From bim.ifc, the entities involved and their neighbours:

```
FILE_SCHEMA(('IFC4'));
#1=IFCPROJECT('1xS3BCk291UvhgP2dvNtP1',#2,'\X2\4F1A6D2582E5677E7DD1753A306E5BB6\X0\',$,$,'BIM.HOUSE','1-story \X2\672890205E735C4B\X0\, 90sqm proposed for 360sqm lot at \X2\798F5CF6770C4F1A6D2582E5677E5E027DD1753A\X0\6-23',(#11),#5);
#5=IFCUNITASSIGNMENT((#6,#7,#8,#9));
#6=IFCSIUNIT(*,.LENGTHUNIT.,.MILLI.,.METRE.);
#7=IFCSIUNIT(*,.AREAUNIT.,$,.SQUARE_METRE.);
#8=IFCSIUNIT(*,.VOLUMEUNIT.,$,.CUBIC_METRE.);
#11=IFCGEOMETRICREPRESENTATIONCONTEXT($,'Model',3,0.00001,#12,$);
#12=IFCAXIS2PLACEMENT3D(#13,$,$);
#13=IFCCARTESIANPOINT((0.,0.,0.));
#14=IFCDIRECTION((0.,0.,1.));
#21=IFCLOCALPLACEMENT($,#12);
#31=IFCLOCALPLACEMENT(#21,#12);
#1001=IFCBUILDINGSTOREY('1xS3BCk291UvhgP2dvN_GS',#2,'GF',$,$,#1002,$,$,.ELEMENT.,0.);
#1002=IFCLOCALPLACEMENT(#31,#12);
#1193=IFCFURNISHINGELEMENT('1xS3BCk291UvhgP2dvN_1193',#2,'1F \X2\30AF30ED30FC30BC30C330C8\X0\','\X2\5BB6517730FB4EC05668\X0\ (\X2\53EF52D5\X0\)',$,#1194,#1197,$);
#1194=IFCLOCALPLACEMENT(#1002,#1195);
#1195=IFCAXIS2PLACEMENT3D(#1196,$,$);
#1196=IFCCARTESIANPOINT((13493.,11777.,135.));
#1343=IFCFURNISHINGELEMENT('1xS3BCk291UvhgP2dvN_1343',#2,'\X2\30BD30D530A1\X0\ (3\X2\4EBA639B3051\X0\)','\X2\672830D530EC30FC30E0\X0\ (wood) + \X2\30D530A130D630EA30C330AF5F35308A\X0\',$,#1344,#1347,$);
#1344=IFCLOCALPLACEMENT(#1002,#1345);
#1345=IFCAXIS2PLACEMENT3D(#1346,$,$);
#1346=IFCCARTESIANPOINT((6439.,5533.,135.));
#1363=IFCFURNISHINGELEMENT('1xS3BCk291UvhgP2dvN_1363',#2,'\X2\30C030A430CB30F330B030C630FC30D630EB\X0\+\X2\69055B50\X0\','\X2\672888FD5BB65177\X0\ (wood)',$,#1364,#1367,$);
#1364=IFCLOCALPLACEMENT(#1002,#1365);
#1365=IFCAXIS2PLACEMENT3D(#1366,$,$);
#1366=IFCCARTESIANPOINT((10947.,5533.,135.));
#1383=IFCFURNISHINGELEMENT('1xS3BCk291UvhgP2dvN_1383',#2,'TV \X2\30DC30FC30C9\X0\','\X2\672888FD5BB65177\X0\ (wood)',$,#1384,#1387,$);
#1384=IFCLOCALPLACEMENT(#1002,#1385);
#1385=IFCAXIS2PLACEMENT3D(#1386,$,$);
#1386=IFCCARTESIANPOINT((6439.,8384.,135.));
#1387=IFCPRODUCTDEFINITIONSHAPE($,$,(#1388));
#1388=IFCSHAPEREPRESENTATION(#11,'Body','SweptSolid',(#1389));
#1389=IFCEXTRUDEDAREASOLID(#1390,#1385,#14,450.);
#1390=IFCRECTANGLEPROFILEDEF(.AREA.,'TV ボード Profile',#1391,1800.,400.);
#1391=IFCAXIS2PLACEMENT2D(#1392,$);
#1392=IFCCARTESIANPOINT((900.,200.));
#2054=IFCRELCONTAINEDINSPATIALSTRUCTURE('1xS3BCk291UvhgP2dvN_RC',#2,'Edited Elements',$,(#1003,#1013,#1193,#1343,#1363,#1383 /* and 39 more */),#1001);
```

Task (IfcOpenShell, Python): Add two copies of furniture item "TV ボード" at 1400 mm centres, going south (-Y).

```python
import numpy as np
import ifcopenshell
import ifcopenshell.api.geometry
import ifcopenshell.api.root
import ifcopenshell.util.element
import ifcopenshell.util.placement

model = ifcopenshell.open("bim.ifc")


def reuse_history(source, copy):
    """copy_class also copies each property set's owner history, people and application; keep the originals."""
    for rel in copy.IsDefinedBy:
        if rel.is_a("IfcRelDefinesByProperties") and (history := rel.RelatingPropertyDefinition.OwnerHistory):
            rel.RelatingPropertyDefinition.OwnerHistory = source.OwnerHistory
            ifcopenshell.util.element.remove_deep2(model, history)


source = model.by_guid("1xS3BCk291UvhgP2dvN_1383")
base = ifcopenshell.util.placement.get_local_placement(source.ObjectPlacement)
step = np.array([0.0, -1.0, 0.0]) * 1400.0

for i in range(1, 3):
    copy = ifcopenshell.api.root.copy_class(model, product=source)
    copy.Representation = ifcopenshell.util.element.copy_deep(
        model, source.Representation, exclude=["IfcGeometricRepresentationContext", "IfcRepresentationMap"]
    )
    reuse_history(source, copy)
    matrix = base.copy()
    matrix[:3, 3] += i * step
    print("added at", matrix[:3, 3].round(3) + 0.0)
    ifcopenshell.api.geometry.edit_object_placement(model, product=copy, matrix=matrix, is_si=False)

model.write("bim_edited.ifc")
```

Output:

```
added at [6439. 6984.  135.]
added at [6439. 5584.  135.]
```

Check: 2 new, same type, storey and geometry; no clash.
